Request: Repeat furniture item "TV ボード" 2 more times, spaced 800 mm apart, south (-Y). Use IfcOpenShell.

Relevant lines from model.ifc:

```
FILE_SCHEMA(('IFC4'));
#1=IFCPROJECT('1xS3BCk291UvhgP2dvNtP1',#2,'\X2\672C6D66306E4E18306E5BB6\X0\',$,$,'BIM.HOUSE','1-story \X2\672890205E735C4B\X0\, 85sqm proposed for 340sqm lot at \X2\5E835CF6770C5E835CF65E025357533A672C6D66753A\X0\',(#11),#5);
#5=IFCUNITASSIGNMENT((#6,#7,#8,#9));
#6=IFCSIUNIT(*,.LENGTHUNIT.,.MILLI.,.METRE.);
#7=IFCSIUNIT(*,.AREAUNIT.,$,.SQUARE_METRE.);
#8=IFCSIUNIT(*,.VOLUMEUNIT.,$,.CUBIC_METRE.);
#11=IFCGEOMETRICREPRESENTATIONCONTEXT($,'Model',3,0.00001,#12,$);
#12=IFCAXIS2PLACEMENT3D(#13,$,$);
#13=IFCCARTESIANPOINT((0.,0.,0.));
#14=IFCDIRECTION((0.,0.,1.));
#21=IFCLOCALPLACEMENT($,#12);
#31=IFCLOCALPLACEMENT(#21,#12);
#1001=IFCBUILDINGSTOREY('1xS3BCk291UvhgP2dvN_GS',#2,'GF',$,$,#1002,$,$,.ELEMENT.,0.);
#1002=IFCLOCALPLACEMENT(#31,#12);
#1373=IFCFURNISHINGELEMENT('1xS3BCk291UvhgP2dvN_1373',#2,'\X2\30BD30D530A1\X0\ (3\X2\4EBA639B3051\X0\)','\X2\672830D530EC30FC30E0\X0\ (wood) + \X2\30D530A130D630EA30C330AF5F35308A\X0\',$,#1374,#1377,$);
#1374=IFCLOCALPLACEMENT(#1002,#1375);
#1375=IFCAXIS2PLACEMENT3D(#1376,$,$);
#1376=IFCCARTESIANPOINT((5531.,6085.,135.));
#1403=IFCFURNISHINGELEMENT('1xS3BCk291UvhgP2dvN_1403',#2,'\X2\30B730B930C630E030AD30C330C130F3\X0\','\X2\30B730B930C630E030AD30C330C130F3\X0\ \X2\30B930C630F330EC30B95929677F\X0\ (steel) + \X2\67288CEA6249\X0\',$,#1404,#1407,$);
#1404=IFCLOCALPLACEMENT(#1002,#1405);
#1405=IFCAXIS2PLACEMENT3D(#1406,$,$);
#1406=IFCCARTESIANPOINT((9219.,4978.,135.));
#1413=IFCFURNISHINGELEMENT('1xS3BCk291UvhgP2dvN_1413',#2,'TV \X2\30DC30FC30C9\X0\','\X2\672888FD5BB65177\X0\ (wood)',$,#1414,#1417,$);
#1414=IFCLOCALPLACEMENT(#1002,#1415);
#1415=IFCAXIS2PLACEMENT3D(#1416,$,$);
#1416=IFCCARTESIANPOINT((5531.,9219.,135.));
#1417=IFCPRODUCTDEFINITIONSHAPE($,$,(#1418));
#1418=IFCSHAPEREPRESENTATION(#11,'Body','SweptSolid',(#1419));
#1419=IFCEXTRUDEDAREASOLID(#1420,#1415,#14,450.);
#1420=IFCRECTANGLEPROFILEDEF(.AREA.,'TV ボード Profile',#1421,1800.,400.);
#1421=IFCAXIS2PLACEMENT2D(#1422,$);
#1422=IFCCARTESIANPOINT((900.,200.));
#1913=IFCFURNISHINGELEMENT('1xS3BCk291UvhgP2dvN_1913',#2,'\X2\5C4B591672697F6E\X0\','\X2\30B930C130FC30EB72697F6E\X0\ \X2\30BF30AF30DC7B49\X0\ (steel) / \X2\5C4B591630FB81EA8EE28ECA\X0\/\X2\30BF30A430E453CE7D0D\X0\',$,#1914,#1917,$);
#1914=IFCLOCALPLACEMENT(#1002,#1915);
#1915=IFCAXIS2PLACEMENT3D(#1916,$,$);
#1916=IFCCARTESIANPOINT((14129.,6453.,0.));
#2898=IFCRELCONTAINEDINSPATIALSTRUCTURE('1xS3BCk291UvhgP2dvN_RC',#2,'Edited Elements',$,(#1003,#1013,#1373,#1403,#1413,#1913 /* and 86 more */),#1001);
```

```python
import numpy as np
import ifcopenshell
import ifcopenshell.api.geometry
import ifcopenshell.api.root
import ifcopenshell.util.element
import ifcopenshell.util.placement

model = ifcopenshell.open("model.ifc")


def reuse_history(source, copy):
    """copy_class also copies each property set's owner history, people and application; keep the originals."""
    for rel in copy.IsDefinedBy:
        if rel.is_a("IfcRelDefinesByProperties") and (history := rel.RelatingPropertyDefinition.OwnerHistory):
            rel.RelatingPropertyDefinition.OwnerHistory = source.OwnerHistory
            ifcopenshell.util.element.remove_deep2(model, history)


source = model.by_guid("1xS3BCk291UvhgP2dvN_1413")
base = ifcopenshell.util.placement.get_local_placement(source.ObjectPlacement)
step = np.array([0.0, -1.0, 0.0]) * 800.0

for i in range(1, 3):
    copy = ifcopenshell.api.root.copy_class(model, product=source)
    copy.Representation = ifcopenshell.util.element.copy_deep(
        model, source.Representation, exclude=["IfcGeometricRepresentationContext", "IfcRepresentationMap"]
    )
    reuse_history(source, copy)
    matrix = base.copy()
    matrix[:3, 3] += i * step
    print("added at", matrix[:3, 3].round(3) + 0.0)
    ifcopenshell.api.geometry.edit_object_placement(model, product=copy, matrix=matrix, is_si=False)

model.write("model_edited.ifc")
```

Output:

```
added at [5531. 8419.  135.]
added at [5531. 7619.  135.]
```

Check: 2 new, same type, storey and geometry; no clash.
